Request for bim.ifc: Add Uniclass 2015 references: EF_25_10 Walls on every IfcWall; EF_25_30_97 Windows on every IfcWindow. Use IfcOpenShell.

First a look at what the model holds.

```python
import ifcopenshell

model = ifcopenshell.open("bim.ifc")
print(model.schema)
print("classifications:", [c.Name for c in model.by_type("IfcClassification")])
for ifc_class in ("IfcDoor", "IfcRoof", "IfcStair", "IfcWall", "IfcWindow"):
    print(ifc_class, len(model.by_type(ifc_class)))
```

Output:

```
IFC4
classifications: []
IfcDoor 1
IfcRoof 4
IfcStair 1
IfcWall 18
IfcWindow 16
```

```python
import ifcopenshell
import ifcopenshell.api.classification

model = ifcopenshell.open("bim.ifc")

system = ifcopenshell.api.classification.add_classification(model, classification="Uniclass 2015")

codes = {
    "IfcWall": ("EF_25_10", "Walls"),
    "IfcWindow": ("EF_25_30_97", "Windows"),
}
for ifc_class, (code, name) in codes.items():
    products = model.by_type(ifc_class)
    ifcopenshell.api.classification.add_reference(
        model, products=products, classification=system, identification=code, name=name
    )
    print(code, len(products))

model.write("bim_edited.ifc")
```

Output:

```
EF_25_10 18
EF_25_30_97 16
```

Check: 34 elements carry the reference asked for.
